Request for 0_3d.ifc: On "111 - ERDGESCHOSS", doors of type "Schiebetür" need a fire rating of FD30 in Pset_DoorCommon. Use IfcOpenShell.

First a look at what the model holds.

```python
import ifcopenshell
import ifcopenshell.util.element

model = ifcopenshell.open("0_3d.ifc")
print(model.schema)
storey = next(s for s in model.by_type("IfcBuildingStorey") if s.Name == "111 - ERDGESCHOSS")
doors = [e for e in ifcopenshell.util.element.get_decomposition(storey) if e.is_a("IfcDoor")]
seen = {}
for e in doors:
    element_type = ifcopenshell.util.element.get_type(e)
    key = (element_type.Name if element_type != e and element_type else None, ifcopenshell.util.element.get_pset(e, "Pset_DoorCommon", "FireRating"))
    seen[key] = seen.get(key, 0) + 1
for (name, value), count in sorted(seen.items(), key=str):
    print(count, "x", name, "|", value)
```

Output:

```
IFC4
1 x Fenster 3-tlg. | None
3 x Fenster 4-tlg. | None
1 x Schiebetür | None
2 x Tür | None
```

```python
import ifcopenshell
import ifcopenshell.api.pset
import ifcopenshell.util.element

model = ifcopenshell.open("0_3d.ifc")

storey = next(s for s in model.by_type("IfcBuildingStorey") if s.Name == "111 - ERDGESCHOSS")
doors = [e for e in ifcopenshell.util.element.get_decomposition(storey) if e.is_a("IfcDoor")]

count = 0
for e in doors:
    element_type = ifcopenshell.util.element.get_type(e)
    if element_type in (None, e) or element_type.Name != "Schiebetür":
        continue
    # add_pset returns the element's existing set when there is one.
    pset = ifcopenshell.api.pset.add_pset(model, product=e, name="Pset_DoorCommon")
    ifcopenshell.api.pset.edit_pset(model, pset=pset, properties={"FireRating": "FD30"})
    count += 1

print(count, "doors updated")

model.write("0_3d_v2.ifc")
```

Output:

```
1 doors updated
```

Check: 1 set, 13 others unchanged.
